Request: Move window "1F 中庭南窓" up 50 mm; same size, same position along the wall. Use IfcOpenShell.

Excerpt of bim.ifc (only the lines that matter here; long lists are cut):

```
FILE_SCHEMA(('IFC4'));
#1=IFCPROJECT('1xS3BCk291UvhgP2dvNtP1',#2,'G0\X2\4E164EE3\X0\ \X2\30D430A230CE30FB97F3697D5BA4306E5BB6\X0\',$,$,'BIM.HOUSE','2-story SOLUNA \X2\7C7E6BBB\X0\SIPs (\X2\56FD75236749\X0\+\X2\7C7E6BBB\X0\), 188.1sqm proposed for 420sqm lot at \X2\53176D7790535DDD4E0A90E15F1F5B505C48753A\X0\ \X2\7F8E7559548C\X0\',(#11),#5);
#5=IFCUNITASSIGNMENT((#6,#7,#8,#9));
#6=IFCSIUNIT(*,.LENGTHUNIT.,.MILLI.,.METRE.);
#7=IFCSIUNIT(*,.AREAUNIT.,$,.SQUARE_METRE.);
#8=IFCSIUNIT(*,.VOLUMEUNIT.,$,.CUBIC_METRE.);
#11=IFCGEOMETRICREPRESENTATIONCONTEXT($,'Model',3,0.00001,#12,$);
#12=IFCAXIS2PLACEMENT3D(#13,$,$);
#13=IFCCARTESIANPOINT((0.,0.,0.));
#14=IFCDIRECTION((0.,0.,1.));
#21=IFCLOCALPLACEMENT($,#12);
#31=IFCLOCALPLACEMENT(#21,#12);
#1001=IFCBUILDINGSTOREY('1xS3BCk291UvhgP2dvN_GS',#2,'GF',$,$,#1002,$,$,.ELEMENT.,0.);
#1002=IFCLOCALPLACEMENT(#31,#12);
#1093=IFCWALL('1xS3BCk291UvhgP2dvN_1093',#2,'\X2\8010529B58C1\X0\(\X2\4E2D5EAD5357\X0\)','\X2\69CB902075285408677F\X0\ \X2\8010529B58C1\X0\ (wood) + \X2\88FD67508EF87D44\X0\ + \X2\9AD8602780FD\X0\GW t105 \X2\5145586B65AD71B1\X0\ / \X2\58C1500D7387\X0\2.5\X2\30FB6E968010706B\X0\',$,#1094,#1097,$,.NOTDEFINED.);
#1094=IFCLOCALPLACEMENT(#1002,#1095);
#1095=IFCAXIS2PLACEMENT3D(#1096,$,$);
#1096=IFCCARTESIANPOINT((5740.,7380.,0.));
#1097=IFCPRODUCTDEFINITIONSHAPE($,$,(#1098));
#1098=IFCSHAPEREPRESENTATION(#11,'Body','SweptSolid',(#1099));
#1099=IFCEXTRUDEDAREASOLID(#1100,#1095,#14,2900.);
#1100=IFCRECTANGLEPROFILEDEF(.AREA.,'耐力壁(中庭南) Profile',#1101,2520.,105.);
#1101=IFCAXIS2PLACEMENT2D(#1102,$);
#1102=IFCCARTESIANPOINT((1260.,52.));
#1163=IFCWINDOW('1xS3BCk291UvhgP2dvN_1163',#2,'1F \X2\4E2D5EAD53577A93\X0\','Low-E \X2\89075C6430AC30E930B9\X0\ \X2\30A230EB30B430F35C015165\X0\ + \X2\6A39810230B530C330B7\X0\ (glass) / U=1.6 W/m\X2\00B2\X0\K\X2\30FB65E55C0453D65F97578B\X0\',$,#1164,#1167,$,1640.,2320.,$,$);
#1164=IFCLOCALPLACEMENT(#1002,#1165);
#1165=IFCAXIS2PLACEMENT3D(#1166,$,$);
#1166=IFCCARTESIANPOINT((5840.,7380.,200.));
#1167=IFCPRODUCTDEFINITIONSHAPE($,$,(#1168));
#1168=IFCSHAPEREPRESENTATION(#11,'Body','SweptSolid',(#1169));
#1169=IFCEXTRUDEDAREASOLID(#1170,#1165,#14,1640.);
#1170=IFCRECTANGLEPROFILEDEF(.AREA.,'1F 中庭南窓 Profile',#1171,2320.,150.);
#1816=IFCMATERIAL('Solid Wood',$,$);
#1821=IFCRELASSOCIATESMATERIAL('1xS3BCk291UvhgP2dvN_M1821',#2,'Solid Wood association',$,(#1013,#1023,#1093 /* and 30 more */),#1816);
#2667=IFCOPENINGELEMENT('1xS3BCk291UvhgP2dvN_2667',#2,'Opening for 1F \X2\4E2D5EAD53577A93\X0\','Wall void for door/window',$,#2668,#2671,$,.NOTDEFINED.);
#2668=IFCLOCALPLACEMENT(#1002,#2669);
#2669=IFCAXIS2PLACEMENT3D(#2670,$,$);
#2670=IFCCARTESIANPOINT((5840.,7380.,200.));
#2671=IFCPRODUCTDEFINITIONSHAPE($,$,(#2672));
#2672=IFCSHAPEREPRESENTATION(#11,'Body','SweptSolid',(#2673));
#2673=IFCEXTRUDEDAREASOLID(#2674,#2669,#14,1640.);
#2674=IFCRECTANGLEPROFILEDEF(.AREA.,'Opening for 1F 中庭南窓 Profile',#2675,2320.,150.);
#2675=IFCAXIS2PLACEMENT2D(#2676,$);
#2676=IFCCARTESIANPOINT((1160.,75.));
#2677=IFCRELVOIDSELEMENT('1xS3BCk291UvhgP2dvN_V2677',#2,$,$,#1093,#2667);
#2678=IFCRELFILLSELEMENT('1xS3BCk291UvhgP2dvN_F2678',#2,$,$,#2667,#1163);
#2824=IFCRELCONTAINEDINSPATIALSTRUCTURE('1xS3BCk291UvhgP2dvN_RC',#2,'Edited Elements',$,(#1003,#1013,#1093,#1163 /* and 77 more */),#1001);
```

```python
import numpy as np
import ifcopenshell
import ifcopenshell.api.geometry
import ifcopenshell.util.placement
import ifcopenshell.util.unit

model = ifcopenshell.open("bim.ifc")
unit_scale = ifcopenshell.util.unit.calculate_unit_scale(model)

window = model.by_guid("1xS3BCk291UvhgP2dvN_1163")
opening = window.FillsVoids[0].RelatingOpeningElement
dz = 0.05 / unit_scale

shift = np.array([0.0, 0.0, dz])
# The window is not placed relative to its opening, so move both.
for product in (opening, window):
    matrix = ifcopenshell.util.placement.get_local_placement(product.ObjectPlacement)
    matrix[:3, 3] += shift
    ifcopenshell.api.geometry.edit_object_placement(model, product=product, matrix=matrix, is_si=False)

print(f"moved by {dz * unit_scale:+.3f} m")

model.write("bim_updated.ifc")
```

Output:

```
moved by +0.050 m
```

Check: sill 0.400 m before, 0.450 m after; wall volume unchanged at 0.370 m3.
